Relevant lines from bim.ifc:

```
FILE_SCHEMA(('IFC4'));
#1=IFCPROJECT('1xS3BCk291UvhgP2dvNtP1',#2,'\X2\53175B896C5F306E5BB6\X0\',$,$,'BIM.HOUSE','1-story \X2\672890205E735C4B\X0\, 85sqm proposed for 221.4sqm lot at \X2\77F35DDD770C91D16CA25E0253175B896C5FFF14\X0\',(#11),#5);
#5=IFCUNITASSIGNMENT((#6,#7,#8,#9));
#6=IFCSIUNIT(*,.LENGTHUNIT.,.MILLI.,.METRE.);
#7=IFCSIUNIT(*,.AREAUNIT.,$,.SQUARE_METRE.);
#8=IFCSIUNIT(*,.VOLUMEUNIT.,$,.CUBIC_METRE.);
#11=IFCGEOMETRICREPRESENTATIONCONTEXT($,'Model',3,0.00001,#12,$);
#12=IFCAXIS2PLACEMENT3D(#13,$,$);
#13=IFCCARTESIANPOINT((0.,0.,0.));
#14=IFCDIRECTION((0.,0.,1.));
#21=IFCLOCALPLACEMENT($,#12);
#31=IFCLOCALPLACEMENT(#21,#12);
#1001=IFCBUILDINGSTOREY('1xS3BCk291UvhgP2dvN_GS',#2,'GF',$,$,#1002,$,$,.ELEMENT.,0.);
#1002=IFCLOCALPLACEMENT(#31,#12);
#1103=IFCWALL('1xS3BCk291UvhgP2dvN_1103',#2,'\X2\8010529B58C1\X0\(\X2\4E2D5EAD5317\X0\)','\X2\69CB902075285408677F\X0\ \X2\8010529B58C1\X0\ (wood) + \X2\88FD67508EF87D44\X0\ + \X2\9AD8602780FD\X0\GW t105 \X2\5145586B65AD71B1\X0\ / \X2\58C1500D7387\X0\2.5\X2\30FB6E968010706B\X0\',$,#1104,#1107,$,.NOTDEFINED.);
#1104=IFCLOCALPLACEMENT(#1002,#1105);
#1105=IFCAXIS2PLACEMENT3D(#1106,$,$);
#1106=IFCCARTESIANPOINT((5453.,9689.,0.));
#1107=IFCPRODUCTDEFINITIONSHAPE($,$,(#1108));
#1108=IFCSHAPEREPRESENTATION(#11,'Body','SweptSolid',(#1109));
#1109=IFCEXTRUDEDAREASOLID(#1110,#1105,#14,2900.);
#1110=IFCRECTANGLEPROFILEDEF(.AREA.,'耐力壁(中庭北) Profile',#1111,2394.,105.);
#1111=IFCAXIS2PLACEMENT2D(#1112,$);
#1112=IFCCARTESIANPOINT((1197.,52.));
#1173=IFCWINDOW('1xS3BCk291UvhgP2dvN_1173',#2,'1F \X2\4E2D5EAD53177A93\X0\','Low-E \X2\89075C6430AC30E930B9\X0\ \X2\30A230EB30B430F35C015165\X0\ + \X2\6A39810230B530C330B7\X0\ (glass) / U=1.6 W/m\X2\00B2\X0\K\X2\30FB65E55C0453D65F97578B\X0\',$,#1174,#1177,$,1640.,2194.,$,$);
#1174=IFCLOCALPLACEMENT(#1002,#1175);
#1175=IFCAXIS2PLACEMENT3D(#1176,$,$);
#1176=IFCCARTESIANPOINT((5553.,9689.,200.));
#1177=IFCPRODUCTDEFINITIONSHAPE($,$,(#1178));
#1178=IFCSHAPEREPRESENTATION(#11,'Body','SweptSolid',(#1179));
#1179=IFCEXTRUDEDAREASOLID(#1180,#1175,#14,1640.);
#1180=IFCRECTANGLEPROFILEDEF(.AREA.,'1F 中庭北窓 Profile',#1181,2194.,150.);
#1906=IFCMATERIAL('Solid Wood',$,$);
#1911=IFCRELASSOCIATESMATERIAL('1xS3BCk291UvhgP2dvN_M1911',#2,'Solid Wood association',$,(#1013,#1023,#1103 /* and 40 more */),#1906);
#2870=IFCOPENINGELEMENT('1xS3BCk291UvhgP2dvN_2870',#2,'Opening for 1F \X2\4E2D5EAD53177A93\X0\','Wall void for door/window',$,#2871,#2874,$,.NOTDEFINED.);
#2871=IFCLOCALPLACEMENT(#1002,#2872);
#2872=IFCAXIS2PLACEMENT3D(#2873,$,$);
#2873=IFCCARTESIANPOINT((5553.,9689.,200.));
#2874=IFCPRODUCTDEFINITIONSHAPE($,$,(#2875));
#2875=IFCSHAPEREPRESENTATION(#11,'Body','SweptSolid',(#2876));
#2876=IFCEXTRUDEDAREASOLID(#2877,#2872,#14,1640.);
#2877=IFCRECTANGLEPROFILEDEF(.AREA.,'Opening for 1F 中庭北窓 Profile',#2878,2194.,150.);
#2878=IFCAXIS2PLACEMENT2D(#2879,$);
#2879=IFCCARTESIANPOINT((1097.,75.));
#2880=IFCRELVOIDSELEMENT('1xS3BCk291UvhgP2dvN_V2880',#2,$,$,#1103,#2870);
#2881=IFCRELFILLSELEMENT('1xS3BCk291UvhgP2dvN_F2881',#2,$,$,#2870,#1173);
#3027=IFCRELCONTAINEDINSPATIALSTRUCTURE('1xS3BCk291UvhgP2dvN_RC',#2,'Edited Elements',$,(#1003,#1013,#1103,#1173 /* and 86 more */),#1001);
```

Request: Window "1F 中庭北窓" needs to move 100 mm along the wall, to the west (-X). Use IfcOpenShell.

```python
import ifcopenshell
import ifcopenshell.api.geometry
import ifcopenshell.util.placement
import ifcopenshell.util.unit

model = ifcopenshell.open("bim.ifc")
unit_scale = ifcopenshell.util.unit.calculate_unit_scale(model)

window = model.by_guid("1xS3BCk291UvhgP2dvN_1173")
opening = window.FillsVoids[0].RelatingOpeningElement
wall = opening.VoidsElements[0].RelatingBuildingElement

wall_matrix = ifcopenshell.util.placement.get_local_placement(wall.ObjectPlacement)
shift = wall_matrix[:3, 0] * -0.1 / unit_scale
before = ifcopenshell.util.placement.get_local_placement(window.ObjectPlacement)[:3, 3].copy()

# The window is not placed relative to its opening, so move both.
for product in (opening, window):
    matrix = ifcopenshell.util.placement.get_local_placement(product.ObjectPlacement)
    matrix[:3, 3] += shift
    ifcopenshell.api.geometry.edit_object_placement(model, product=product, matrix=matrix, is_si=False)

after = ifcopenshell.util.placement.get_local_placement(window.ObjectPlacement)[:3, 3]
print("window moved by", (after - before).round(3) + 0.0)

model.write("bim-out.ifc")
```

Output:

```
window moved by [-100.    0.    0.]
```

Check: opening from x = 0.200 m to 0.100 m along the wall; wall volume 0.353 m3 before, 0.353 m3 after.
